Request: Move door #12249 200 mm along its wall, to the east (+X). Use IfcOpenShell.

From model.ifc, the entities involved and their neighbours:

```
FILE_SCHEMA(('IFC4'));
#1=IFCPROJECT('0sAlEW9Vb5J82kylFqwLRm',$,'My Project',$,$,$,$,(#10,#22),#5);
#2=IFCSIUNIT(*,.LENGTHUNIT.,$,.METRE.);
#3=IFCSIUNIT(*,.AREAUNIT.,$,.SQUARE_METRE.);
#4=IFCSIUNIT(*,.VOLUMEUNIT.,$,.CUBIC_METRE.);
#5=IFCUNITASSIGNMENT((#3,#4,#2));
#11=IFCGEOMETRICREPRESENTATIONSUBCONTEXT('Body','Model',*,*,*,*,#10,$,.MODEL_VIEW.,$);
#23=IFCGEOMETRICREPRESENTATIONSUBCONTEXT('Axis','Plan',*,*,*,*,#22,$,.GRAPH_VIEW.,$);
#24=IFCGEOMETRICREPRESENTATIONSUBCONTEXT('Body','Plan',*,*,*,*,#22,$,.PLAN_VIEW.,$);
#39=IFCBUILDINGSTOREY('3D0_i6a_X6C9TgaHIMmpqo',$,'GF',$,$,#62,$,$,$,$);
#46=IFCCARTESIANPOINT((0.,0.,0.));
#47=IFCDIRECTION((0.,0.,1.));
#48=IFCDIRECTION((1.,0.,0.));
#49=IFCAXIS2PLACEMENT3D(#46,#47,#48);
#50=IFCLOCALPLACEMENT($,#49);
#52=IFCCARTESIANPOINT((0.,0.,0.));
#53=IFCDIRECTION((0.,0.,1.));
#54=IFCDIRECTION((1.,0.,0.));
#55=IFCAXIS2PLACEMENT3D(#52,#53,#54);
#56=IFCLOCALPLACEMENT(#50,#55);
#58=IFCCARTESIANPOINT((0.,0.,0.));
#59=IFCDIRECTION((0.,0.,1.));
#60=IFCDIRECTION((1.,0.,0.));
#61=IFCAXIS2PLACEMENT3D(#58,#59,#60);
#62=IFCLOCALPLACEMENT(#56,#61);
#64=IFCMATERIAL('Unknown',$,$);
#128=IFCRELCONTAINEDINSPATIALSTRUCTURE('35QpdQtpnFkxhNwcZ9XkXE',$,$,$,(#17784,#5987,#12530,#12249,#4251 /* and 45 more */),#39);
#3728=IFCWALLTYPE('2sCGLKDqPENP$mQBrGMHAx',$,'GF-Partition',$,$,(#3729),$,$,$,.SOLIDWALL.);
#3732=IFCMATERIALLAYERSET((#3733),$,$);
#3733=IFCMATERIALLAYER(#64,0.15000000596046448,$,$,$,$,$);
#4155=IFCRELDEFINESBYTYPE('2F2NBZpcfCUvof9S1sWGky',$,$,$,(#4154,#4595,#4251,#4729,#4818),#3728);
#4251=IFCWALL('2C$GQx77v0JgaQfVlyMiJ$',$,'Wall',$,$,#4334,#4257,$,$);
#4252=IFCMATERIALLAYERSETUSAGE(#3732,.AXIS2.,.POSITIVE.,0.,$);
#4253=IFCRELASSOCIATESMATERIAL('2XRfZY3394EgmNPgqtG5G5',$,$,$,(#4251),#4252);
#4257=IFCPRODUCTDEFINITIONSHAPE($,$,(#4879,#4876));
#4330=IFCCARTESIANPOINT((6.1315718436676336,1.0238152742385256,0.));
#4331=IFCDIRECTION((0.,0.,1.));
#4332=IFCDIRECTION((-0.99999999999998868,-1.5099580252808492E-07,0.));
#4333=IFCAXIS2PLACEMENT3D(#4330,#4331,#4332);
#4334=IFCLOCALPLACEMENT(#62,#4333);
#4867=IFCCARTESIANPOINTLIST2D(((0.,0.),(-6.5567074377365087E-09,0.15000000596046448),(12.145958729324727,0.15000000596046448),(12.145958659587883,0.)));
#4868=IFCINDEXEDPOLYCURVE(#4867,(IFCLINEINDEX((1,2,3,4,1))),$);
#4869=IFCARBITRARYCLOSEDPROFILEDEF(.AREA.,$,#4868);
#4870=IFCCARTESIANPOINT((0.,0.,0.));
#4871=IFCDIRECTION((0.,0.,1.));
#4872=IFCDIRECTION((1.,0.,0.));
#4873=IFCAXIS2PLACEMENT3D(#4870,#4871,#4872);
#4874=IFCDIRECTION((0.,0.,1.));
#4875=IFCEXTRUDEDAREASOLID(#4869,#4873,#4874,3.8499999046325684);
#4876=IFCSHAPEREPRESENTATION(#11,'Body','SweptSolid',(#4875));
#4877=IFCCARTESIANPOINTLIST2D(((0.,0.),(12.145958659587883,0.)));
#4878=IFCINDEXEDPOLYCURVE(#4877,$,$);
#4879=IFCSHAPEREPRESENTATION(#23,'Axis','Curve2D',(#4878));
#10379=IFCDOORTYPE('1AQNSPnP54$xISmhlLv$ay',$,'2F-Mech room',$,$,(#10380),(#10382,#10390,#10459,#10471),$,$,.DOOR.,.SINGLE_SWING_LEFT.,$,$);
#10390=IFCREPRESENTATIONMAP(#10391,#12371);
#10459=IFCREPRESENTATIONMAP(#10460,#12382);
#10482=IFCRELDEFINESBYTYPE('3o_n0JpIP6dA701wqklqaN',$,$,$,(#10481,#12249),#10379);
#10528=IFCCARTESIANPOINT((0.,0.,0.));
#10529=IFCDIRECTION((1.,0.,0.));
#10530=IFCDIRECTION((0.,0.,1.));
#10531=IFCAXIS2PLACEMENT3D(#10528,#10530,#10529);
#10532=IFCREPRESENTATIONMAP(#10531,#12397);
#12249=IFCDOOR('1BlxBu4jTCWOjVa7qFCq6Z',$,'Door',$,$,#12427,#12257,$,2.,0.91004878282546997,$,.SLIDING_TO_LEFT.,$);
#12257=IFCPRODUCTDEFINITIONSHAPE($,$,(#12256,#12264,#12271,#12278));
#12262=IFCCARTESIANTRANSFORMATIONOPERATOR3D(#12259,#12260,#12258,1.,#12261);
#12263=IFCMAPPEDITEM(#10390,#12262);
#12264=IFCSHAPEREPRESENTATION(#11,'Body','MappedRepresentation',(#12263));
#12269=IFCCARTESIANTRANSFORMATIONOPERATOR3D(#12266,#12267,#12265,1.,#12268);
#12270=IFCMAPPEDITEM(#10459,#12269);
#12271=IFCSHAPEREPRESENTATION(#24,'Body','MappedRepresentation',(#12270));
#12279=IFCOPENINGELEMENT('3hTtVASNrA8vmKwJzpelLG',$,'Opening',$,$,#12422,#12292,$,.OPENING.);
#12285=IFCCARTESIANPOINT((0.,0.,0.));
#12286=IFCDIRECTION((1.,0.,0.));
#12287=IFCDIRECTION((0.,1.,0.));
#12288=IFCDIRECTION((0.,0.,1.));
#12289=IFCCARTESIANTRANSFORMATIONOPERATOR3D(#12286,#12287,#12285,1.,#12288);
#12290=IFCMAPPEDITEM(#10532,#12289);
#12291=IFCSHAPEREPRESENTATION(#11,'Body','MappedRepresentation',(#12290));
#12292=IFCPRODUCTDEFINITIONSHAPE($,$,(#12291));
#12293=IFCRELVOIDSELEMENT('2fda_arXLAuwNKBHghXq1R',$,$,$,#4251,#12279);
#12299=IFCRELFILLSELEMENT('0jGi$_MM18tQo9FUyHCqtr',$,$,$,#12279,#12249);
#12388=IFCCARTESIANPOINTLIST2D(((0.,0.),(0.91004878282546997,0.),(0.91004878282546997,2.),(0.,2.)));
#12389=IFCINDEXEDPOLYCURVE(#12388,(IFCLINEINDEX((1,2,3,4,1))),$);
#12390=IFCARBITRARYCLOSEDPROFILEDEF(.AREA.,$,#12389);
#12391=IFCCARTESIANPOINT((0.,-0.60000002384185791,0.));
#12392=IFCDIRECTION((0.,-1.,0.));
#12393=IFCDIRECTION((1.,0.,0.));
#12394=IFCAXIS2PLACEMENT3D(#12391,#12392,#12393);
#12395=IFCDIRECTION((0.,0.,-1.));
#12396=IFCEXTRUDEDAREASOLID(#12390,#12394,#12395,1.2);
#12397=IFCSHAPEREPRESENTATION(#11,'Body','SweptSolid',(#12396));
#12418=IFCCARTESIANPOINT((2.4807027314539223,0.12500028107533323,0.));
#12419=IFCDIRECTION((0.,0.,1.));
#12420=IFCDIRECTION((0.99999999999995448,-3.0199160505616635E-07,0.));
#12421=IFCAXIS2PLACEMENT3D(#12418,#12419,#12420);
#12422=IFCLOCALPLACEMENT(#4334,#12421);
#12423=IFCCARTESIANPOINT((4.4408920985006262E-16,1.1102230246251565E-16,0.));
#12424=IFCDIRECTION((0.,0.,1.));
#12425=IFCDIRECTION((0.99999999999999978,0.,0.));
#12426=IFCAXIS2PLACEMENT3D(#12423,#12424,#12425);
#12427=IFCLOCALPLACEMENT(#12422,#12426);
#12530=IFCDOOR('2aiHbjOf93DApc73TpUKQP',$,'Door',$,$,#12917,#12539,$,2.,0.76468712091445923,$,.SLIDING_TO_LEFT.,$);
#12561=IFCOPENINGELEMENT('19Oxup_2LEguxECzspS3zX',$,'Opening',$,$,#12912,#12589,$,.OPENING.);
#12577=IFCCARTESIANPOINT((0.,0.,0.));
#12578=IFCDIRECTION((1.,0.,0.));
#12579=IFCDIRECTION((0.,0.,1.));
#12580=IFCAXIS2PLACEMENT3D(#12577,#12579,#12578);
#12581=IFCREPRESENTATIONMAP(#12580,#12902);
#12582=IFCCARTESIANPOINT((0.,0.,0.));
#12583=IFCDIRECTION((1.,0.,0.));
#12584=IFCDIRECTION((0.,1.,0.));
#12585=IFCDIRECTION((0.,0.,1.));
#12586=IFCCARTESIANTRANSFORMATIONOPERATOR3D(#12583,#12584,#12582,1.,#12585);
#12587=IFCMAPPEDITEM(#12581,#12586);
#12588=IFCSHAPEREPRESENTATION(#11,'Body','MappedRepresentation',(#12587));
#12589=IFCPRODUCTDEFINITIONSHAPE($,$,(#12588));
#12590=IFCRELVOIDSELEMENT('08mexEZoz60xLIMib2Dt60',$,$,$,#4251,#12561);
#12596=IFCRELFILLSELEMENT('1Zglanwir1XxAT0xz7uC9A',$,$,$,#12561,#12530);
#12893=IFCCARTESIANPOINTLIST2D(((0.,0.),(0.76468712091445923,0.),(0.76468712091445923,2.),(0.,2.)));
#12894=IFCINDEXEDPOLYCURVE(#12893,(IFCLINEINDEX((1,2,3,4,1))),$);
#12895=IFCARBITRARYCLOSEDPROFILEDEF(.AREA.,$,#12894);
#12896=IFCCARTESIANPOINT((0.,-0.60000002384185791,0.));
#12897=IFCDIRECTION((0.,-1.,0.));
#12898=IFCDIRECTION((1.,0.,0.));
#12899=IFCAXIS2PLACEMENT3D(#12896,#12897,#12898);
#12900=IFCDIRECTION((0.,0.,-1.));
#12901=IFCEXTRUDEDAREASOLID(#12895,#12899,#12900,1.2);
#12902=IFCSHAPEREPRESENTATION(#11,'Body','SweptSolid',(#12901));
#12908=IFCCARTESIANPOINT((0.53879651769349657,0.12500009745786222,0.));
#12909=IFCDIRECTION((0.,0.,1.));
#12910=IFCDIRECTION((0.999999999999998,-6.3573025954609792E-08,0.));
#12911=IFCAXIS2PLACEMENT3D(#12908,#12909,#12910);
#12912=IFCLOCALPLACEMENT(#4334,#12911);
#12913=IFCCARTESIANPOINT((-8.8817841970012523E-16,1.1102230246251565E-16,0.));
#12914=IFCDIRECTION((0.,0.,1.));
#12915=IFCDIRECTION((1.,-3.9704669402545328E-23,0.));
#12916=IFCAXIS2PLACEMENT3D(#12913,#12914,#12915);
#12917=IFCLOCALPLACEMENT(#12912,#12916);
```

```python
import ifcopenshell
import ifcopenshell.api.geometry
import ifcopenshell.util.placement
import ifcopenshell.util.unit

model = ifcopenshell.open("model.ifc")
unit_scale = ifcopenshell.util.unit.calculate_unit_scale(model)

door = model.by_id(12249)
opening = door.FillsVoids[0].RelatingOpeningElement
wall = opening.VoidsElements[0].RelatingBuildingElement

wall_matrix = ifcopenshell.util.placement.get_local_placement(wall.ObjectPlacement)
shift = wall_matrix[:3, 0] * -0.2 / unit_scale
before = ifcopenshell.util.placement.get_local_placement(door.ObjectPlacement)[:3, 3].copy()

# The door is placed relative to its opening, so it follows when the opening moves.
matrix = ifcopenshell.util.placement.get_local_placement(opening.ObjectPlacement)
matrix[:3, 3] += shift
ifcopenshell.api.geometry.edit_object_placement(
    model, product=opening, matrix=matrix, is_si=False, should_transform_children=True
)

after = ifcopenshell.util.placement.get_local_placement(door.ObjectPlacement)[:3, 3]
print("door moved by", (after - before).round(3) + 0.0)

model.write("model_edited.ifc")
```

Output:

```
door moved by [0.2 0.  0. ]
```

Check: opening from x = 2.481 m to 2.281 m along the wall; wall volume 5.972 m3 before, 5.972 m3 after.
